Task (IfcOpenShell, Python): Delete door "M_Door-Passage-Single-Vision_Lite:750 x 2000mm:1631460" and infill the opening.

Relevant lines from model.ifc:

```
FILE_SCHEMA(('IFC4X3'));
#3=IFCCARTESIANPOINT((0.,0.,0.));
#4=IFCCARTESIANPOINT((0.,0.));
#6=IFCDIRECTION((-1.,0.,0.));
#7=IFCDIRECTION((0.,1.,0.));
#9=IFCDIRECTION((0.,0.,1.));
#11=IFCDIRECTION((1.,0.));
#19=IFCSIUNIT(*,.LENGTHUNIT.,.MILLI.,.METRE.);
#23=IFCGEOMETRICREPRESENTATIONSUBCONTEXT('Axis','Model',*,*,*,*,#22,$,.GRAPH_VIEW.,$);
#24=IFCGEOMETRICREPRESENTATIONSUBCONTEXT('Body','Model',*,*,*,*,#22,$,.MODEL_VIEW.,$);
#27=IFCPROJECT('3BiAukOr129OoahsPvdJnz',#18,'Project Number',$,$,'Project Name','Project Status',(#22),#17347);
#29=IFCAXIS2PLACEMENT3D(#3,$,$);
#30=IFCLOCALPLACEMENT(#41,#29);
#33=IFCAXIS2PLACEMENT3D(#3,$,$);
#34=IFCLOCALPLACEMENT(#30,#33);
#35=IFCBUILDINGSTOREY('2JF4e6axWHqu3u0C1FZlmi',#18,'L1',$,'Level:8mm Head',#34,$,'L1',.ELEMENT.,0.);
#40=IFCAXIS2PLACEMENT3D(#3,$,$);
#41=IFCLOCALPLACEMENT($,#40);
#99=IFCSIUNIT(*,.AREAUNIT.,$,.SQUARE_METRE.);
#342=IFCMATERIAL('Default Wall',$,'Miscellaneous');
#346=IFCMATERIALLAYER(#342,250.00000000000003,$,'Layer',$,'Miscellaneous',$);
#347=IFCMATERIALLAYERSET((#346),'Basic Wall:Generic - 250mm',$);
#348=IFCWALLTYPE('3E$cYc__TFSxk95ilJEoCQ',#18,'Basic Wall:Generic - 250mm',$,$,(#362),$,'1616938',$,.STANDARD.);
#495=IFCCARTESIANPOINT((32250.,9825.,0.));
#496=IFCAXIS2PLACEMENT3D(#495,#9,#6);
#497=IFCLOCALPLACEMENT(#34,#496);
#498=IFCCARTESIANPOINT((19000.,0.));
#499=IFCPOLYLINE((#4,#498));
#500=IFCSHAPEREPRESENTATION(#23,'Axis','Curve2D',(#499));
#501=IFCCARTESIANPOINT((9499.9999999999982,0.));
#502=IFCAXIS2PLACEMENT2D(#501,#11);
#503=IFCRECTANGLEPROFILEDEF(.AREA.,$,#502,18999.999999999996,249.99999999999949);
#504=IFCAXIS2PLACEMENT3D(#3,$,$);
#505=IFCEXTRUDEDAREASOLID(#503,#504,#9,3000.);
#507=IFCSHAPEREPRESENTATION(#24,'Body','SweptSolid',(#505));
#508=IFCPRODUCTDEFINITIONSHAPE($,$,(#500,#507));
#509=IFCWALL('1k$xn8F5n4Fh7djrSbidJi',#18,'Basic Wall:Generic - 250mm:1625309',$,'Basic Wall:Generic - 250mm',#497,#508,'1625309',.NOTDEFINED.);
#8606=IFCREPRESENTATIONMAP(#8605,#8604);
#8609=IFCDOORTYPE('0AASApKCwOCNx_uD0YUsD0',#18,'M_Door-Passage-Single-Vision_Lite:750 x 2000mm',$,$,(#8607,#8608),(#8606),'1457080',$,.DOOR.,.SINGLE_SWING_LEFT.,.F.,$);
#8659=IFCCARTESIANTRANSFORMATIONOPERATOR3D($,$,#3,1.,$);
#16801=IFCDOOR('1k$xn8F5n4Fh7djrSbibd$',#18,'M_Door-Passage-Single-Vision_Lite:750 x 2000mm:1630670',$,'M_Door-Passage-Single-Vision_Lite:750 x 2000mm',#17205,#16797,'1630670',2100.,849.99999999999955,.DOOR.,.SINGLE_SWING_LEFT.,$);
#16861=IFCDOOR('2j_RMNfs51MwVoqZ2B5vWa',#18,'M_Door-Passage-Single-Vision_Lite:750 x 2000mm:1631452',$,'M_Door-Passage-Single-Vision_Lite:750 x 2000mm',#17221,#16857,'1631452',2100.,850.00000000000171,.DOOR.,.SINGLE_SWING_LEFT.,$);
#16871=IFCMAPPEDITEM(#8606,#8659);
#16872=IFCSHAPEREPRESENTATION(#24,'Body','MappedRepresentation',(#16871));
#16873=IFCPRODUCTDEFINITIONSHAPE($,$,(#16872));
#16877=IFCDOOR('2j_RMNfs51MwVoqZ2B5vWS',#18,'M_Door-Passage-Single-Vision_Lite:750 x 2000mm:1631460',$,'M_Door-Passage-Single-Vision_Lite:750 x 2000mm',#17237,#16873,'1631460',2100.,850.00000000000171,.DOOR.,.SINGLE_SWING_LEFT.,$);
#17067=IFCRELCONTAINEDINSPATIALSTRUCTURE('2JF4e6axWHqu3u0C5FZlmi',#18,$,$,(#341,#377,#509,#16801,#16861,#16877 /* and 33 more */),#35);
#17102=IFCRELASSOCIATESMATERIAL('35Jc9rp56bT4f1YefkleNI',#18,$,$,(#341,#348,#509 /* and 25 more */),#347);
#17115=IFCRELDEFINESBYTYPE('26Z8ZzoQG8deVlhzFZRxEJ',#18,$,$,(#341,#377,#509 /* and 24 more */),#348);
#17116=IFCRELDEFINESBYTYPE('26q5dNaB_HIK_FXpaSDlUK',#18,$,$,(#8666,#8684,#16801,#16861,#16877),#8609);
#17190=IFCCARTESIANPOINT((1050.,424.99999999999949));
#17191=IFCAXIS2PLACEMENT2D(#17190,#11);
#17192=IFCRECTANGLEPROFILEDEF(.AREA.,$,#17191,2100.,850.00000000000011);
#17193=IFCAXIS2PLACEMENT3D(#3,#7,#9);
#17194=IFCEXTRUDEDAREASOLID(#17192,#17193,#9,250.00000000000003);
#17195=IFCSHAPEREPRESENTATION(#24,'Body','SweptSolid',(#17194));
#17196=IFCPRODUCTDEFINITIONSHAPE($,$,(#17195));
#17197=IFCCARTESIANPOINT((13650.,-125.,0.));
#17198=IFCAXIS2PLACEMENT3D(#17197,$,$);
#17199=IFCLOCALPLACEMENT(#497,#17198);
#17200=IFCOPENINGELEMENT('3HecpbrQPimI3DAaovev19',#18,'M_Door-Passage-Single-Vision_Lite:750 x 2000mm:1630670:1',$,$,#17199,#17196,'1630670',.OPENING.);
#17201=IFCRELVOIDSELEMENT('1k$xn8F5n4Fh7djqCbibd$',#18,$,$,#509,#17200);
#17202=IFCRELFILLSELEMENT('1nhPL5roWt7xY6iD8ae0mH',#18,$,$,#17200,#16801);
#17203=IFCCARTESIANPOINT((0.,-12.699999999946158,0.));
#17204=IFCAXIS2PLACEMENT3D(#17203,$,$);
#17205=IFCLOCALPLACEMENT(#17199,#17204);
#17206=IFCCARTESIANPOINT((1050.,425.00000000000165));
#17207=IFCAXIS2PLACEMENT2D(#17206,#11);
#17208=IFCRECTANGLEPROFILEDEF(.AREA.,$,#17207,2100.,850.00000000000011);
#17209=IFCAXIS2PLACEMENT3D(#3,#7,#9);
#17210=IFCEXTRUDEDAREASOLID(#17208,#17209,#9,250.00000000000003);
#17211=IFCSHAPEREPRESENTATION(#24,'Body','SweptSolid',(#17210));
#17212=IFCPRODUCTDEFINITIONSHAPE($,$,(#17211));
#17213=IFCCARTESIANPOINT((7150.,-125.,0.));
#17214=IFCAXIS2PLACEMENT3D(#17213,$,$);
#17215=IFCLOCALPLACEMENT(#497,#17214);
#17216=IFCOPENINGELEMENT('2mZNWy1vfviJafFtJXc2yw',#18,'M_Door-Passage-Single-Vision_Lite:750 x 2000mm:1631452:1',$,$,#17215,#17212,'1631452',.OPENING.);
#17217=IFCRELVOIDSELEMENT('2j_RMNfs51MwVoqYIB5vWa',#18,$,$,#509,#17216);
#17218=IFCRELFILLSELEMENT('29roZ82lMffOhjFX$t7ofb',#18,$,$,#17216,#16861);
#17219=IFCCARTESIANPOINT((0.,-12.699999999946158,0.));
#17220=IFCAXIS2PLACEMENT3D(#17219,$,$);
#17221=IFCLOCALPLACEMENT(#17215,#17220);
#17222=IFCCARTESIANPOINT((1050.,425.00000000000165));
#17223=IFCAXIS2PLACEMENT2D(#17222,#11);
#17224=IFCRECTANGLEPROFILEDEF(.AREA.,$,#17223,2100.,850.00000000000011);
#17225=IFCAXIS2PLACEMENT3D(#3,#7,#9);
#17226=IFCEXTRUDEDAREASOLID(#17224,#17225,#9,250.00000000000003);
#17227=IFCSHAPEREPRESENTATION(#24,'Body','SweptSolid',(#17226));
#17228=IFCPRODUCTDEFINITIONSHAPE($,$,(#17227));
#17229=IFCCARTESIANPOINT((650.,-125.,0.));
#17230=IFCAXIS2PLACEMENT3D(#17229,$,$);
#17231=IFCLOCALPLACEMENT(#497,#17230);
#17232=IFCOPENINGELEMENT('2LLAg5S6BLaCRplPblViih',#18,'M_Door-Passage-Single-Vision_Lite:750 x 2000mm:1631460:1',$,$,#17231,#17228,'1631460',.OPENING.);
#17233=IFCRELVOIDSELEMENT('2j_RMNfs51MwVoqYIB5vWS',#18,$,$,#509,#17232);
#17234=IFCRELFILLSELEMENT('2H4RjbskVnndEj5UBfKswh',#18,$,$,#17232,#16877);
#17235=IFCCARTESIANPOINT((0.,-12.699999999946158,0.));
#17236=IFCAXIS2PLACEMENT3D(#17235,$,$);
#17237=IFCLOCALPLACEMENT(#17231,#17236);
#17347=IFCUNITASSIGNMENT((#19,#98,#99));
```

```python
import ifcopenshell
import ifcopenshell.api.feature
import ifcopenshell.api.root
import ifcopenshell.geom
import ifcopenshell.util.shape

model = ifcopenshell.open("model.ifc")
settings = ifcopenshell.geom.settings()


def volume(element):
    """Net volume in cubic metres, openings subtracted."""
    shape = ifcopenshell.geom.create_shape(settings, element)
    return ifcopenshell.util.shape.get_volume(shape.geometry)


door = model.by_guid("2j_RMNfs51MwVoqZ2B5vWS")
opening = door.FillsVoids[0].RelatingOpeningElement
wall = opening.VoidsElements[0].RelatingBuildingElement
before = volume(wall)

ifcopenshell.api.root.remove_product(model, product=door)
ifcopenshell.api.feature.remove_feature(model, feature=opening)

after = volume(wall)

print(f"wall volume {before:.3f} -> {after:.3f} m3")

model.write("model_rev.ifc")
```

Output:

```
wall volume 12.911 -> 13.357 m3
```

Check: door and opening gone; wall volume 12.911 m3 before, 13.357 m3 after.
